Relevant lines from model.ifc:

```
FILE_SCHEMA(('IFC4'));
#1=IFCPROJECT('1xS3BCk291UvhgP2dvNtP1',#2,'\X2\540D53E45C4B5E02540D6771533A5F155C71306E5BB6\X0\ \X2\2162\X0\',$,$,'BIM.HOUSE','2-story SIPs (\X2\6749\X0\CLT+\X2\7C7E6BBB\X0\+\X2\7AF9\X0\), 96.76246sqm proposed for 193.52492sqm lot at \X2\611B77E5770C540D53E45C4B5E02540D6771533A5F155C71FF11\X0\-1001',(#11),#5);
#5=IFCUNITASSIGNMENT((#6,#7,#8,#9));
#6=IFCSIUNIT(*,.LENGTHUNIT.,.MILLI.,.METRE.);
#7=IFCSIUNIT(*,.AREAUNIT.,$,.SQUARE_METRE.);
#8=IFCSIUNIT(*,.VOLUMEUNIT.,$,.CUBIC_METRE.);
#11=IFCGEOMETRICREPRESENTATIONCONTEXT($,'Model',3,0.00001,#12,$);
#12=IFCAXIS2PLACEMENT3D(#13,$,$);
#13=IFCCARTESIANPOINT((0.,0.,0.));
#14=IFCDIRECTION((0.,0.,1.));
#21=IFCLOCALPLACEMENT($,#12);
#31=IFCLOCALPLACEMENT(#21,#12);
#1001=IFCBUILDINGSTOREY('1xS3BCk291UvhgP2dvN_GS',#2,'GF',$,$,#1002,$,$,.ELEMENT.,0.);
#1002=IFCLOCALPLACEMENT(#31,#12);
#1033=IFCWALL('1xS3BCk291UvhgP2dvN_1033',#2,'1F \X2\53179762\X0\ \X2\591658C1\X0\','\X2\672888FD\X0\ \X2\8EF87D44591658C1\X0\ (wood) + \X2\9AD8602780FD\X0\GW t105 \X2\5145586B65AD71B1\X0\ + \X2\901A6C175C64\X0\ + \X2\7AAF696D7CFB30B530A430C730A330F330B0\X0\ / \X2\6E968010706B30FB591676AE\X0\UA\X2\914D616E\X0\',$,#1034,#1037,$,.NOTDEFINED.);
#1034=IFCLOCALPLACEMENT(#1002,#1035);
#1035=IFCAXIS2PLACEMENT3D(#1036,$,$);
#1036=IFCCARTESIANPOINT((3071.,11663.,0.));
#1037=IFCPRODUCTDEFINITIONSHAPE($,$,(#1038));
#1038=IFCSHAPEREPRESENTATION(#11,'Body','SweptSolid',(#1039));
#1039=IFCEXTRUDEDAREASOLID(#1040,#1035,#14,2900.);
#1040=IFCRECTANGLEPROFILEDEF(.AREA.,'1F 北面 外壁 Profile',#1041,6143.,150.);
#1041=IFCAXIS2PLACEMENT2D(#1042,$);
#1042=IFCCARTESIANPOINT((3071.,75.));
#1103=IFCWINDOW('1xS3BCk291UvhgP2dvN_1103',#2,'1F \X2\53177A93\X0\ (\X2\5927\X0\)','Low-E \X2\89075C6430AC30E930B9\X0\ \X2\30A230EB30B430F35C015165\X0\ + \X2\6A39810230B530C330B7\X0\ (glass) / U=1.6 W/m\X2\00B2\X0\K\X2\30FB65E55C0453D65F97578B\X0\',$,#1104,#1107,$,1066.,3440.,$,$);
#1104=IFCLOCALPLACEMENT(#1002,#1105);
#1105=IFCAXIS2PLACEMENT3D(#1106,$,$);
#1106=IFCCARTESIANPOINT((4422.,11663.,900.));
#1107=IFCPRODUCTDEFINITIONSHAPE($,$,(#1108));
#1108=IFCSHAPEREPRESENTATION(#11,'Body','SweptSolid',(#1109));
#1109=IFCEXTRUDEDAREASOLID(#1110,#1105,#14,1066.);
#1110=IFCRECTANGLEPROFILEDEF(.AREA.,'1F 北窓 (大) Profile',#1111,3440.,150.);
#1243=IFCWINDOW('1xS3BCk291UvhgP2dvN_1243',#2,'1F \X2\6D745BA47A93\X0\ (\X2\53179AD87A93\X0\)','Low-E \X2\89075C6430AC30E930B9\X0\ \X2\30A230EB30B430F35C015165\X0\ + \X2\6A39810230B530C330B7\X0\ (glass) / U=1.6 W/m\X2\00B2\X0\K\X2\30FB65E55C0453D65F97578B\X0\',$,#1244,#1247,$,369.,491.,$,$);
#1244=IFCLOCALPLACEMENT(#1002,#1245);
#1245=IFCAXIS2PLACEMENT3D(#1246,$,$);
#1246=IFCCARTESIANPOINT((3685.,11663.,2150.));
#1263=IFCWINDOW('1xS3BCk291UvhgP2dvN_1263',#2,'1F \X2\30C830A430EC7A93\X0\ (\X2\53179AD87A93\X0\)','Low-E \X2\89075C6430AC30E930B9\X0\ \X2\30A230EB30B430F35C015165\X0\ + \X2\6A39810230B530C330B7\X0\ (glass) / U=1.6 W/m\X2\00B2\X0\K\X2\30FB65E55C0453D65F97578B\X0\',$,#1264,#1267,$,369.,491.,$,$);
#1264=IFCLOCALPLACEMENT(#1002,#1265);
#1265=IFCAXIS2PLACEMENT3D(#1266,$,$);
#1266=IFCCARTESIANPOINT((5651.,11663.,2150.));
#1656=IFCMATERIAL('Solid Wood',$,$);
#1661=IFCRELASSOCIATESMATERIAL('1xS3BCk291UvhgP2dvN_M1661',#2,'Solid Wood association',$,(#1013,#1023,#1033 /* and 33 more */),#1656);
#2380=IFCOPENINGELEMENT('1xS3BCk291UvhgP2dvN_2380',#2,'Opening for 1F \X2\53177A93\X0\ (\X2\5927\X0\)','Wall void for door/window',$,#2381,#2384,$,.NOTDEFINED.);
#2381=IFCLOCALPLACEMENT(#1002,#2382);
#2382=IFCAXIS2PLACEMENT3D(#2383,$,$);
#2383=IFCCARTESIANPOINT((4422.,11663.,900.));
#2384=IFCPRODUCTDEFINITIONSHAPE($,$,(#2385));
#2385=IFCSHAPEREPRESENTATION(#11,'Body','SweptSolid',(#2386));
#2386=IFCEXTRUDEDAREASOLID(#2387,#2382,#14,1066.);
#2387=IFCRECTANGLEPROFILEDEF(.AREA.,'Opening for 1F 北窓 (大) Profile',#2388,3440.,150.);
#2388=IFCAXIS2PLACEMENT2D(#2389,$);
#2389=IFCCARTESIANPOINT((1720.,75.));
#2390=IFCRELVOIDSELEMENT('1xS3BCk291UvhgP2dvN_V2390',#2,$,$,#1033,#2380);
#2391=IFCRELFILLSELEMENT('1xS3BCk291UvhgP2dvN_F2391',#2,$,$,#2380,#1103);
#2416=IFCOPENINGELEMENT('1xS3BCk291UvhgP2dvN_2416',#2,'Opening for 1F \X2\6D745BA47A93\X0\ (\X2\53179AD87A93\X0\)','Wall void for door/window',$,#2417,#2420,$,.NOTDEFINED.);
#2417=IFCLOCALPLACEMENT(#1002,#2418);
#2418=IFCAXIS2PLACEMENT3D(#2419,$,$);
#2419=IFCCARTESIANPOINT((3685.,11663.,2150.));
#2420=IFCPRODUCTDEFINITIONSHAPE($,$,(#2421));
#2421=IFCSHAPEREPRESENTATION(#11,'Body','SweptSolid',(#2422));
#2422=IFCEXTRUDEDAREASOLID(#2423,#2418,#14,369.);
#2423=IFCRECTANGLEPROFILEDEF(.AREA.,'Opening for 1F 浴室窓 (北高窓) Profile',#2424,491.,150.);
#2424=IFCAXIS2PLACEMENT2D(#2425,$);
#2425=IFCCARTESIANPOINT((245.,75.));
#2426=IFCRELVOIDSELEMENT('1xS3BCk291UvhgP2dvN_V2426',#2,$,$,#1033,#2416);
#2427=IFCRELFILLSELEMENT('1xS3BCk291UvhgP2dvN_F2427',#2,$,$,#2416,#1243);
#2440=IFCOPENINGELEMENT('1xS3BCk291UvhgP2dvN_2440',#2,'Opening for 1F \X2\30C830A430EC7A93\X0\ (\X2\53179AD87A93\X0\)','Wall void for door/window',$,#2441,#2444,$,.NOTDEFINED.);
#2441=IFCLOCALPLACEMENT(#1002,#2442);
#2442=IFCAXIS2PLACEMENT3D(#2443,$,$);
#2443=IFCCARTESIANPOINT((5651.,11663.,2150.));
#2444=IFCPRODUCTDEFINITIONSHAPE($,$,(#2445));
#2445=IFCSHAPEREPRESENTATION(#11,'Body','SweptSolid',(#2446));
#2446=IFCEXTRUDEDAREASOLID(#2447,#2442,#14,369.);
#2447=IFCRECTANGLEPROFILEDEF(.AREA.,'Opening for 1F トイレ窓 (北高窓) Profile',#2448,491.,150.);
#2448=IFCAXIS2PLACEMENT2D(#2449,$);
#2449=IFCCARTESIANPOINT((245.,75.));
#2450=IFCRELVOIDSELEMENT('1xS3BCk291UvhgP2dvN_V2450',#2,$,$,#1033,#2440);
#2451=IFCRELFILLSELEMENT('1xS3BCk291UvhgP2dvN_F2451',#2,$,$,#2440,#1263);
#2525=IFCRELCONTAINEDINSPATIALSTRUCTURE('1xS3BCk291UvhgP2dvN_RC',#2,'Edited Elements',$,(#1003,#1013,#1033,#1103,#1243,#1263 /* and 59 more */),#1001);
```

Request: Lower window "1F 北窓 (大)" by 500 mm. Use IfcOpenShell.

```python
import numpy as np
import ifcopenshell
import ifcopenshell.api.geometry
import ifcopenshell.util.placement
import ifcopenshell.util.unit

model = ifcopenshell.open("model.ifc")
unit_scale = ifcopenshell.util.unit.calculate_unit_scale(model)

window = model.by_guid("1xS3BCk291UvhgP2dvN_1103")
opening = window.FillsVoids[0].RelatingOpeningElement
dz = -500.0

shift = np.array([0.0, 0.0, dz])
# The window is not placed relative to its opening, so move both.
for product in (opening, window):
    matrix = ifcopenshell.util.placement.get_local_placement(product.ObjectPlacement)
    matrix[:3, 3] += shift
    ifcopenshell.api.geometry.edit_object_placement(model, product=product, matrix=matrix, is_si=False)

print(f"moved by {dz * unit_scale:+.3f} m")

model.write("model_updated.ifc")
```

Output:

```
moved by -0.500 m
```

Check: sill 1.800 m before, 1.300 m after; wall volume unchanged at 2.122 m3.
